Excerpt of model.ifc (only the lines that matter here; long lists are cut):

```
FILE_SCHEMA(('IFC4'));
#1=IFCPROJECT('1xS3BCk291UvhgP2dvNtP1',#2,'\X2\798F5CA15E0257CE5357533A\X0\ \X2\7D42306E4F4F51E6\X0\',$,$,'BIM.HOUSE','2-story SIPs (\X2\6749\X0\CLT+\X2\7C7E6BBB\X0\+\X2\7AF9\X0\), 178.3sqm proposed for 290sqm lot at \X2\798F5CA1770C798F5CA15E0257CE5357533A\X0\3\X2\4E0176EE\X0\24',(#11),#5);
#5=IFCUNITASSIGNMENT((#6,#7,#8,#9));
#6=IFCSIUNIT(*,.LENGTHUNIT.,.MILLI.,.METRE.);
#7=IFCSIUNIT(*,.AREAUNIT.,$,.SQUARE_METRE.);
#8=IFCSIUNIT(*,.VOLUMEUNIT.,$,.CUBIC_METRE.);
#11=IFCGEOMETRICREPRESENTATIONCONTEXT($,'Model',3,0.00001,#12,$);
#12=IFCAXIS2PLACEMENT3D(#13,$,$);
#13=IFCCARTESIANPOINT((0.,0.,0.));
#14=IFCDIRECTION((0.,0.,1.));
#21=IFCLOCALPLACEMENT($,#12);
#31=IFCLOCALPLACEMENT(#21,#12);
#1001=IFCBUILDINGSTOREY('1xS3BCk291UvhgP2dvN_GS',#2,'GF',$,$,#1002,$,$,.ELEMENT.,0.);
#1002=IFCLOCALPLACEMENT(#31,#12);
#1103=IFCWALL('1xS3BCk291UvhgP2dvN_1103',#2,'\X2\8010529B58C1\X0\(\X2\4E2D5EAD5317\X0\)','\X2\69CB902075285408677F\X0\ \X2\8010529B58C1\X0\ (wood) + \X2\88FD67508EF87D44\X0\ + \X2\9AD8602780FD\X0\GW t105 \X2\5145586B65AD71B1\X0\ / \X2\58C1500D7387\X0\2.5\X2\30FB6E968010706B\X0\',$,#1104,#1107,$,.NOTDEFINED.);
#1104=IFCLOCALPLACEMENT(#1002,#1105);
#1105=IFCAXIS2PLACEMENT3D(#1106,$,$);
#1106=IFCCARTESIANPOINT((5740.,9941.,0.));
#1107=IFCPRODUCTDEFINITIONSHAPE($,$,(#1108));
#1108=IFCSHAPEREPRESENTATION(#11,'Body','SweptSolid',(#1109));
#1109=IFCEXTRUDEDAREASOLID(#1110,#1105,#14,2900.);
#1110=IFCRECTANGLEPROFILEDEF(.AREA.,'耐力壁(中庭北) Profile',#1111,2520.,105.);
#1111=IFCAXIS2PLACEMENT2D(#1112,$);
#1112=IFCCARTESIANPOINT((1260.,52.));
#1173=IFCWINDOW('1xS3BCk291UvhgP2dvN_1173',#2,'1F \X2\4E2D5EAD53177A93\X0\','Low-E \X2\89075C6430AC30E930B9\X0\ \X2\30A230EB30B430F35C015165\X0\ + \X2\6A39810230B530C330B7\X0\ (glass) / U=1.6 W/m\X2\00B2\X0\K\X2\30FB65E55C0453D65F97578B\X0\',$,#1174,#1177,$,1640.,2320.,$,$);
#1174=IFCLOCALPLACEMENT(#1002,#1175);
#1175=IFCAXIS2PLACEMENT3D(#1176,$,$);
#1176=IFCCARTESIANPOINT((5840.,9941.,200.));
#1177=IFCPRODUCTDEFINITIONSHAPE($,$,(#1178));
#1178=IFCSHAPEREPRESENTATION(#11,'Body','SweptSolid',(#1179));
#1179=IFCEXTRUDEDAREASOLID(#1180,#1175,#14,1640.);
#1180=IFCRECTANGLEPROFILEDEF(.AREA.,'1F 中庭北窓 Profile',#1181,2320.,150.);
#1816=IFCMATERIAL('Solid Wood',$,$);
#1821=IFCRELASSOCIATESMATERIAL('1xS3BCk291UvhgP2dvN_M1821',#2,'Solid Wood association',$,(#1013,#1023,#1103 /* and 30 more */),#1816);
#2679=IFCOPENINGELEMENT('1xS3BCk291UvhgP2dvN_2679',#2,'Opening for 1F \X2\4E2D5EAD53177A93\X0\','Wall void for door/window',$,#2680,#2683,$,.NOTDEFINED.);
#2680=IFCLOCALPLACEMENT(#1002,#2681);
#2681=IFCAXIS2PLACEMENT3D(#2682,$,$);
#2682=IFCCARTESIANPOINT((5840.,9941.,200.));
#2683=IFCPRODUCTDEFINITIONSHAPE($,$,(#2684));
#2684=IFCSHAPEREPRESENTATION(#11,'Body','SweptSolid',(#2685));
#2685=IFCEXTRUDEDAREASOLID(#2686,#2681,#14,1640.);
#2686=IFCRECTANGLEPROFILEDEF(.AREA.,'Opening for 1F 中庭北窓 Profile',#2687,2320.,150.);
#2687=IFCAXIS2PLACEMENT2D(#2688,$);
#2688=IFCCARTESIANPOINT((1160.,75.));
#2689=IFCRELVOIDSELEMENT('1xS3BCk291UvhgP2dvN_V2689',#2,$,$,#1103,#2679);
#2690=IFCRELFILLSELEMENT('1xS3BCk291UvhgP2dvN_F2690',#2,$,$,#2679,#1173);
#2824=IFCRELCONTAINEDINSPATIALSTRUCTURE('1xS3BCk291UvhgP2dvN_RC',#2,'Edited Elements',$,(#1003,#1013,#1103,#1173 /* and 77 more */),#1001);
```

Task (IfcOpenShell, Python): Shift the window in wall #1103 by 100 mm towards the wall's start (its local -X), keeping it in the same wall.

```python
import ifcopenshell
import ifcopenshell.api.geometry
import ifcopenshell.util.placement
import ifcopenshell.util.unit

model = ifcopenshell.open("model.ifc")
unit_scale = ifcopenshell.util.unit.calculate_unit_scale(model)

window = model.by_guid("1xS3BCk291UvhgP2dvN_1173")
opening = window.FillsVoids[0].RelatingOpeningElement
wall = opening.VoidsElements[0].RelatingBuildingElement

wall_matrix = ifcopenshell.util.placement.get_local_placement(wall.ObjectPlacement)
shift = wall_matrix[:3, 0] * -0.1 / unit_scale
before = ifcopenshell.util.placement.get_local_placement(window.ObjectPlacement)[:3, 3].copy()

# The window is not placed relative to its opening, so move both.
for product in (opening, window):
    matrix = ifcopenshell.util.placement.get_local_placement(product.ObjectPlacement)
    matrix[:3, 3] += shift
    ifcopenshell.api.geometry.edit_object_placement(model, product=product, matrix=matrix, is_si=False)

after = ifcopenshell.util.placement.get_local_placement(window.ObjectPlacement)[:3, 3]
print("window moved by", (after - before).round(3) + 0.0)

model.write("model_updated.ifc")
```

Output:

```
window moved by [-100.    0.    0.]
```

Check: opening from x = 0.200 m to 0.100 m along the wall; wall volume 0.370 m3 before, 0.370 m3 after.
